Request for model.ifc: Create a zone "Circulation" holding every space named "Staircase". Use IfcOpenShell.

First a look at what the model holds.

```python
import ifcopenshell

model = ifcopenshell.open("model.ifc")
print(model.schema)
seen = {}
for space in model.by_type("IfcSpace"):
    seen[space.LongName] = seen.get(space.LongName, 0) + 1
for name, count in sorted(seen.items(), key=str):
    print(count, "x", name)
print("zones:", [z.Name for z in model.by_type("IfcZone")][:20])
```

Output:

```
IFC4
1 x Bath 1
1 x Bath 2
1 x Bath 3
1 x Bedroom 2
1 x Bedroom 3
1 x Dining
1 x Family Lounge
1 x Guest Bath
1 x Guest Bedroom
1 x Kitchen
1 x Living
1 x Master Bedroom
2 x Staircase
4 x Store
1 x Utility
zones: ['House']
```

```python
import ifcopenshell
import ifcopenshell.api.group
import ifcopenshell.api.root

model = ifcopenshell.open("model.ifc")

names = {"Staircase"}
spaces = [s for s in model.by_type("IfcSpace") if s.LongName in names]

zone = ifcopenshell.api.root.create_entity(model, ifc_class="IfcZone", name="Circulation")
ifcopenshell.api.group.assign_group(model, products=spaces, group=zone)
print(len(spaces), "spaces in", zone.Name)

model.write("model-out.ifc")
```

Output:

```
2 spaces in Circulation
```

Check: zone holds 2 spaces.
